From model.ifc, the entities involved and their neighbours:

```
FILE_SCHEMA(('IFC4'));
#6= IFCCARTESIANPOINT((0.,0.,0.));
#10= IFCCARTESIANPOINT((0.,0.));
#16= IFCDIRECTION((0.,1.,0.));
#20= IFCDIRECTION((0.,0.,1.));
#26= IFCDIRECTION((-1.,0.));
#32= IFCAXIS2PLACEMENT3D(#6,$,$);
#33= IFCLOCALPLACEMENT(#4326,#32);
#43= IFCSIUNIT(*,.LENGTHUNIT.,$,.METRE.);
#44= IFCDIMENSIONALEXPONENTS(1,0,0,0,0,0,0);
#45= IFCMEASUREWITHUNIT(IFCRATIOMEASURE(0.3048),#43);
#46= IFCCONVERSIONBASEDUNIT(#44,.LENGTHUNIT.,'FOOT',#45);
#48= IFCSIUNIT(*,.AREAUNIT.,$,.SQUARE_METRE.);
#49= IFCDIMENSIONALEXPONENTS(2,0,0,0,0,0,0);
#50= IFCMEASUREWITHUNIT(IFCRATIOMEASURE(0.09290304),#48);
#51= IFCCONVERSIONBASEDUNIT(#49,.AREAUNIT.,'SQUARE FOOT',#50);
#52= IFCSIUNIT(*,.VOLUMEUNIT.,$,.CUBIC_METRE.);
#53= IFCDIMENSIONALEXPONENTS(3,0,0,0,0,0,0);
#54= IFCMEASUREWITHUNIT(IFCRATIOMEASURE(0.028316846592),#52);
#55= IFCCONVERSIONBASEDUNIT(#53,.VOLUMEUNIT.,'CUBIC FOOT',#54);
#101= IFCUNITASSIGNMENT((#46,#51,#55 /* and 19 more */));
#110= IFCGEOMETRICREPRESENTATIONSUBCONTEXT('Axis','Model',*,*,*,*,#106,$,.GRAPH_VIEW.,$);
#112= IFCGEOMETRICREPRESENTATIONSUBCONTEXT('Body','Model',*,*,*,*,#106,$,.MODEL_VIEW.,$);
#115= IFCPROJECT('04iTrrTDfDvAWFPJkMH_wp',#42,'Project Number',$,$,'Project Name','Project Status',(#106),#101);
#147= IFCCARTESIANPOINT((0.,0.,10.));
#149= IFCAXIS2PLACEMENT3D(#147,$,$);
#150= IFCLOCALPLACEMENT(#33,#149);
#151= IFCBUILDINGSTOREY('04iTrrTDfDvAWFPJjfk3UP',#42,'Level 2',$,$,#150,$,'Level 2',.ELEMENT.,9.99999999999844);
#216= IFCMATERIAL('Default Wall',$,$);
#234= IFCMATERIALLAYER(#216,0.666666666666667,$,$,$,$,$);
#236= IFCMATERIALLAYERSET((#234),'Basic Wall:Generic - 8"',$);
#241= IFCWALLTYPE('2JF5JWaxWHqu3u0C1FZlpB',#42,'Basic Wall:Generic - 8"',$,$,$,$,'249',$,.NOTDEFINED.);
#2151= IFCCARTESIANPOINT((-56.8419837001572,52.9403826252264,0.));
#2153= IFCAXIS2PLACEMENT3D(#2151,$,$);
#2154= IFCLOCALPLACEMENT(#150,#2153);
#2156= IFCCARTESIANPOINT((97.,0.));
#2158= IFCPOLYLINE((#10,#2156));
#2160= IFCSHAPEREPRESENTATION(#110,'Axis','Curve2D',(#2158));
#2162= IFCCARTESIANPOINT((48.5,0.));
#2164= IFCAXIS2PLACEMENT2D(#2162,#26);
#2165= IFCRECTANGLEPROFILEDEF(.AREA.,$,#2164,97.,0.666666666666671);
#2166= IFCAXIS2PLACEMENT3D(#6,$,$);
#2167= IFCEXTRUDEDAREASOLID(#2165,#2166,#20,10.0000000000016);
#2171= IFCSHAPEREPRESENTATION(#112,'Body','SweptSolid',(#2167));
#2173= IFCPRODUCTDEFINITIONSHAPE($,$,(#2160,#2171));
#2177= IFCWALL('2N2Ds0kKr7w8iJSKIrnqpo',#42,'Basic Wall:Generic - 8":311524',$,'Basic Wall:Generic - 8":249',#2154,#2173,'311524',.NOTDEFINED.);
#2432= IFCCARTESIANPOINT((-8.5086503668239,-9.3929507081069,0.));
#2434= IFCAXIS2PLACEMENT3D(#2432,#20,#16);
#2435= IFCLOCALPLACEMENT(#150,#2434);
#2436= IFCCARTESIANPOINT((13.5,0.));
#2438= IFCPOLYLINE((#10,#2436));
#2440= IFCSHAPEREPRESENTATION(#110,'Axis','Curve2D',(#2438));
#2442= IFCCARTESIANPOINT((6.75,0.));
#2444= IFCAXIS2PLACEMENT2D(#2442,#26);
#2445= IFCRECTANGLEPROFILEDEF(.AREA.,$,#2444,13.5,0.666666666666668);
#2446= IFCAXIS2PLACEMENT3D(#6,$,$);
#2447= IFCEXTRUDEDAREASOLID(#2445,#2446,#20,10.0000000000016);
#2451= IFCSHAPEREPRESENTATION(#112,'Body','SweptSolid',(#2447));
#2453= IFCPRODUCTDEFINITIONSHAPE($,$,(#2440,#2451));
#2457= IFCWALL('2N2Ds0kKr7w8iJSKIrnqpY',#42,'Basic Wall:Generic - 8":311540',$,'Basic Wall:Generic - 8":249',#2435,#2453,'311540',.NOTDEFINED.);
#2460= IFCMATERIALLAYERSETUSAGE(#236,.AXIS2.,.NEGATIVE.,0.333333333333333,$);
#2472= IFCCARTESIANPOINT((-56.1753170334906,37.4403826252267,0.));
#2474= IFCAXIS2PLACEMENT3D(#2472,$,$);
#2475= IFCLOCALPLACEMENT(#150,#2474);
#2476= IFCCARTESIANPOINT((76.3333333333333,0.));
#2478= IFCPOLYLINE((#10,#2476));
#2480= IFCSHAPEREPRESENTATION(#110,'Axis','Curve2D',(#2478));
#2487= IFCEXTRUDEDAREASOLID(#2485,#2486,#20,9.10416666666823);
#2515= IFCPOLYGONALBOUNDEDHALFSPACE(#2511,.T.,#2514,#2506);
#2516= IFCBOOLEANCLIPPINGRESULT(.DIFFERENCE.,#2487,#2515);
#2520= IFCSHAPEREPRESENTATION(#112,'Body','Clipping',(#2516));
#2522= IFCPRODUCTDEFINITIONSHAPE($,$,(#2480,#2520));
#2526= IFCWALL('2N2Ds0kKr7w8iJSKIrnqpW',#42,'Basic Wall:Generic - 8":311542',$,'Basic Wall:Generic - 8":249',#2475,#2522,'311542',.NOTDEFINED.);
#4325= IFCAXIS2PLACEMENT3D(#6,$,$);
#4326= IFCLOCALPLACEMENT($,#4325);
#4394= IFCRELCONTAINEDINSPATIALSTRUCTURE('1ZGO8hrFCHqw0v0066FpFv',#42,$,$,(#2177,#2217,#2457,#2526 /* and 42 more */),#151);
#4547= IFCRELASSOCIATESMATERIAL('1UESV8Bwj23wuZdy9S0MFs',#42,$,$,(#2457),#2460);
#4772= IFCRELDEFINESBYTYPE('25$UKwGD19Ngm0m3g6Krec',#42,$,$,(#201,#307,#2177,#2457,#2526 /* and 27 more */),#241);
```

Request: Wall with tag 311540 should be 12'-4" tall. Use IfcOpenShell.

```python
import ifcopenshell
import ifcopenshell.geom
import ifcopenshell.util.representation
import ifcopenshell.util.shape
import ifcopenshell.util.unit

model = ifcopenshell.open("model.ifc")
unit_scale = ifcopenshell.util.unit.calculate_unit_scale(model)
settings = ifcopenshell.geom.settings()


def volume(element):
    """Net volume in cubic metres, openings subtracted."""
    shape = ifcopenshell.geom.create_shape(settings, element)
    return ifcopenshell.util.shape.get_volume(shape.geometry)


wall = model.by_guid("2N2Ds0kKr7w8iJSKIrnqpY")
before = volume(wall)

body = ifcopenshell.util.representation.get_representation(wall, "Model", "Body")
solid = body.Items[0]
old_height = solid.Depth
solid.Depth = 148 * 0.0254 / unit_scale
after = volume(wall)

print(f"height {old_height:g} -> {solid.Depth:g}, volume {before:.3f} -> {after:.3f} m3")

model.write("model_updated.ifc")
```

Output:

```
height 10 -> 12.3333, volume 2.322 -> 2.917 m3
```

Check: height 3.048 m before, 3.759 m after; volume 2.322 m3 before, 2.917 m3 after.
